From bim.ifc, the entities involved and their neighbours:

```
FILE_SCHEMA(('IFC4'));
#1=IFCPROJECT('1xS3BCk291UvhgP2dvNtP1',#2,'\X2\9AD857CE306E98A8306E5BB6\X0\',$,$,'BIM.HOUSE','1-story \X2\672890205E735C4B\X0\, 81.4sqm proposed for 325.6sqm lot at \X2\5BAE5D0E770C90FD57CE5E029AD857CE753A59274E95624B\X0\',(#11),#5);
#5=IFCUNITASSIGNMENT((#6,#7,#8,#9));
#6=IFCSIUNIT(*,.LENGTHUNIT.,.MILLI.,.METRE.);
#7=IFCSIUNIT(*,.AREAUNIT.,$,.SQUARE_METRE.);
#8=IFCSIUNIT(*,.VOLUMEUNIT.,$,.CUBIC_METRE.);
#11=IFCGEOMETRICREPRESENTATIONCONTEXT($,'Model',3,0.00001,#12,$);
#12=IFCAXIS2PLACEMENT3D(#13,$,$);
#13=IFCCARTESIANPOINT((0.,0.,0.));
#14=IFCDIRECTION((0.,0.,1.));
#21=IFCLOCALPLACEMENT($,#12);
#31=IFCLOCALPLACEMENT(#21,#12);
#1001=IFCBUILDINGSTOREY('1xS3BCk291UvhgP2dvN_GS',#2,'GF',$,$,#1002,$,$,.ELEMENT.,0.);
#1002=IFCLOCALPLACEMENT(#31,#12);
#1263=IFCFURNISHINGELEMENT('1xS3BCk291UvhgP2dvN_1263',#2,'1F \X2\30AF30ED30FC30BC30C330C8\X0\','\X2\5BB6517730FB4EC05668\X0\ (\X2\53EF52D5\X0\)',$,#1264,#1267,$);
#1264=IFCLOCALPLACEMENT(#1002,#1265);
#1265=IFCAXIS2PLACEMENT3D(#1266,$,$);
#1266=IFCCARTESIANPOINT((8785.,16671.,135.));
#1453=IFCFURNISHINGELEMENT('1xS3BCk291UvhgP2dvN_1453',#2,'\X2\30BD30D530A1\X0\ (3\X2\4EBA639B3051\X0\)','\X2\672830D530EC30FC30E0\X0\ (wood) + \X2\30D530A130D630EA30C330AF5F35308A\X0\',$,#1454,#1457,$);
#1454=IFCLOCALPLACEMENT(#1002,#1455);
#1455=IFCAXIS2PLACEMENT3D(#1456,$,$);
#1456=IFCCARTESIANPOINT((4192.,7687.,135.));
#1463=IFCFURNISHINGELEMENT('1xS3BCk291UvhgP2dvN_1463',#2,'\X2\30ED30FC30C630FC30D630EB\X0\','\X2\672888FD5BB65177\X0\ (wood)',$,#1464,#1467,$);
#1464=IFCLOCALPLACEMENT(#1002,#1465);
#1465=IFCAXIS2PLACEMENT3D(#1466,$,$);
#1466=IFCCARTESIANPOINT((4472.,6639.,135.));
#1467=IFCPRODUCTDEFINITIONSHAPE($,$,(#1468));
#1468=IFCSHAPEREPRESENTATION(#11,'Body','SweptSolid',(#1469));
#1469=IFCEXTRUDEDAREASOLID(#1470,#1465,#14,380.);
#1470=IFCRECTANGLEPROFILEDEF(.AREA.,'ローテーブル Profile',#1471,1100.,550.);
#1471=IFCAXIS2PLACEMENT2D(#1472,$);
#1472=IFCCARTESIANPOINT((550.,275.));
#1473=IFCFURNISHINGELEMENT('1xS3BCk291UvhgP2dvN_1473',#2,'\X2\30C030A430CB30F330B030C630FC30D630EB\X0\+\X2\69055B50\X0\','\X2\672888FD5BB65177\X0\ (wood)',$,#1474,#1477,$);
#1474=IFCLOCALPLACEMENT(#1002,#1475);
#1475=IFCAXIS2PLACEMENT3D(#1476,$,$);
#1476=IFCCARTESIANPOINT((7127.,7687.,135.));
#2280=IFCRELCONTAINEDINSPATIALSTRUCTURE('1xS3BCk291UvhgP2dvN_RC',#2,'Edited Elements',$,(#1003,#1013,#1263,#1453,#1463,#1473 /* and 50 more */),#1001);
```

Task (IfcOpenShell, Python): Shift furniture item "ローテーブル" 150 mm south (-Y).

```python
import ifcopenshell
import ifcopenshell.api.geometry
import ifcopenshell.util.placement
import ifcopenshell.util.unit

model = ifcopenshell.open("bim.ifc")
unit_scale = ifcopenshell.util.unit.calculate_unit_scale(model)

item = model.by_guid("1xS3BCk291UvhgP2dvN_1463")
matrix = ifcopenshell.util.placement.get_local_placement(item.ObjectPlacement)
matrix[1, 3] -= 0.15 / unit_scale
ifcopenshell.api.geometry.edit_object_placement(model, product=item, matrix=matrix, is_si=False)

print(ifcopenshell.util.placement.get_local_placement(item.ObjectPlacement).round(3) + 0.0)

model.write("bim_v2.ifc")
```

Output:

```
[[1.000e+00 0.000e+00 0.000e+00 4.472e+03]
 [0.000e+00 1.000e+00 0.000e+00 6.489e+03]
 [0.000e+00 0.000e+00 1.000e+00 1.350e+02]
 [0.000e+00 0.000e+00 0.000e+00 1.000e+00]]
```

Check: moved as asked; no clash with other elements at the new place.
